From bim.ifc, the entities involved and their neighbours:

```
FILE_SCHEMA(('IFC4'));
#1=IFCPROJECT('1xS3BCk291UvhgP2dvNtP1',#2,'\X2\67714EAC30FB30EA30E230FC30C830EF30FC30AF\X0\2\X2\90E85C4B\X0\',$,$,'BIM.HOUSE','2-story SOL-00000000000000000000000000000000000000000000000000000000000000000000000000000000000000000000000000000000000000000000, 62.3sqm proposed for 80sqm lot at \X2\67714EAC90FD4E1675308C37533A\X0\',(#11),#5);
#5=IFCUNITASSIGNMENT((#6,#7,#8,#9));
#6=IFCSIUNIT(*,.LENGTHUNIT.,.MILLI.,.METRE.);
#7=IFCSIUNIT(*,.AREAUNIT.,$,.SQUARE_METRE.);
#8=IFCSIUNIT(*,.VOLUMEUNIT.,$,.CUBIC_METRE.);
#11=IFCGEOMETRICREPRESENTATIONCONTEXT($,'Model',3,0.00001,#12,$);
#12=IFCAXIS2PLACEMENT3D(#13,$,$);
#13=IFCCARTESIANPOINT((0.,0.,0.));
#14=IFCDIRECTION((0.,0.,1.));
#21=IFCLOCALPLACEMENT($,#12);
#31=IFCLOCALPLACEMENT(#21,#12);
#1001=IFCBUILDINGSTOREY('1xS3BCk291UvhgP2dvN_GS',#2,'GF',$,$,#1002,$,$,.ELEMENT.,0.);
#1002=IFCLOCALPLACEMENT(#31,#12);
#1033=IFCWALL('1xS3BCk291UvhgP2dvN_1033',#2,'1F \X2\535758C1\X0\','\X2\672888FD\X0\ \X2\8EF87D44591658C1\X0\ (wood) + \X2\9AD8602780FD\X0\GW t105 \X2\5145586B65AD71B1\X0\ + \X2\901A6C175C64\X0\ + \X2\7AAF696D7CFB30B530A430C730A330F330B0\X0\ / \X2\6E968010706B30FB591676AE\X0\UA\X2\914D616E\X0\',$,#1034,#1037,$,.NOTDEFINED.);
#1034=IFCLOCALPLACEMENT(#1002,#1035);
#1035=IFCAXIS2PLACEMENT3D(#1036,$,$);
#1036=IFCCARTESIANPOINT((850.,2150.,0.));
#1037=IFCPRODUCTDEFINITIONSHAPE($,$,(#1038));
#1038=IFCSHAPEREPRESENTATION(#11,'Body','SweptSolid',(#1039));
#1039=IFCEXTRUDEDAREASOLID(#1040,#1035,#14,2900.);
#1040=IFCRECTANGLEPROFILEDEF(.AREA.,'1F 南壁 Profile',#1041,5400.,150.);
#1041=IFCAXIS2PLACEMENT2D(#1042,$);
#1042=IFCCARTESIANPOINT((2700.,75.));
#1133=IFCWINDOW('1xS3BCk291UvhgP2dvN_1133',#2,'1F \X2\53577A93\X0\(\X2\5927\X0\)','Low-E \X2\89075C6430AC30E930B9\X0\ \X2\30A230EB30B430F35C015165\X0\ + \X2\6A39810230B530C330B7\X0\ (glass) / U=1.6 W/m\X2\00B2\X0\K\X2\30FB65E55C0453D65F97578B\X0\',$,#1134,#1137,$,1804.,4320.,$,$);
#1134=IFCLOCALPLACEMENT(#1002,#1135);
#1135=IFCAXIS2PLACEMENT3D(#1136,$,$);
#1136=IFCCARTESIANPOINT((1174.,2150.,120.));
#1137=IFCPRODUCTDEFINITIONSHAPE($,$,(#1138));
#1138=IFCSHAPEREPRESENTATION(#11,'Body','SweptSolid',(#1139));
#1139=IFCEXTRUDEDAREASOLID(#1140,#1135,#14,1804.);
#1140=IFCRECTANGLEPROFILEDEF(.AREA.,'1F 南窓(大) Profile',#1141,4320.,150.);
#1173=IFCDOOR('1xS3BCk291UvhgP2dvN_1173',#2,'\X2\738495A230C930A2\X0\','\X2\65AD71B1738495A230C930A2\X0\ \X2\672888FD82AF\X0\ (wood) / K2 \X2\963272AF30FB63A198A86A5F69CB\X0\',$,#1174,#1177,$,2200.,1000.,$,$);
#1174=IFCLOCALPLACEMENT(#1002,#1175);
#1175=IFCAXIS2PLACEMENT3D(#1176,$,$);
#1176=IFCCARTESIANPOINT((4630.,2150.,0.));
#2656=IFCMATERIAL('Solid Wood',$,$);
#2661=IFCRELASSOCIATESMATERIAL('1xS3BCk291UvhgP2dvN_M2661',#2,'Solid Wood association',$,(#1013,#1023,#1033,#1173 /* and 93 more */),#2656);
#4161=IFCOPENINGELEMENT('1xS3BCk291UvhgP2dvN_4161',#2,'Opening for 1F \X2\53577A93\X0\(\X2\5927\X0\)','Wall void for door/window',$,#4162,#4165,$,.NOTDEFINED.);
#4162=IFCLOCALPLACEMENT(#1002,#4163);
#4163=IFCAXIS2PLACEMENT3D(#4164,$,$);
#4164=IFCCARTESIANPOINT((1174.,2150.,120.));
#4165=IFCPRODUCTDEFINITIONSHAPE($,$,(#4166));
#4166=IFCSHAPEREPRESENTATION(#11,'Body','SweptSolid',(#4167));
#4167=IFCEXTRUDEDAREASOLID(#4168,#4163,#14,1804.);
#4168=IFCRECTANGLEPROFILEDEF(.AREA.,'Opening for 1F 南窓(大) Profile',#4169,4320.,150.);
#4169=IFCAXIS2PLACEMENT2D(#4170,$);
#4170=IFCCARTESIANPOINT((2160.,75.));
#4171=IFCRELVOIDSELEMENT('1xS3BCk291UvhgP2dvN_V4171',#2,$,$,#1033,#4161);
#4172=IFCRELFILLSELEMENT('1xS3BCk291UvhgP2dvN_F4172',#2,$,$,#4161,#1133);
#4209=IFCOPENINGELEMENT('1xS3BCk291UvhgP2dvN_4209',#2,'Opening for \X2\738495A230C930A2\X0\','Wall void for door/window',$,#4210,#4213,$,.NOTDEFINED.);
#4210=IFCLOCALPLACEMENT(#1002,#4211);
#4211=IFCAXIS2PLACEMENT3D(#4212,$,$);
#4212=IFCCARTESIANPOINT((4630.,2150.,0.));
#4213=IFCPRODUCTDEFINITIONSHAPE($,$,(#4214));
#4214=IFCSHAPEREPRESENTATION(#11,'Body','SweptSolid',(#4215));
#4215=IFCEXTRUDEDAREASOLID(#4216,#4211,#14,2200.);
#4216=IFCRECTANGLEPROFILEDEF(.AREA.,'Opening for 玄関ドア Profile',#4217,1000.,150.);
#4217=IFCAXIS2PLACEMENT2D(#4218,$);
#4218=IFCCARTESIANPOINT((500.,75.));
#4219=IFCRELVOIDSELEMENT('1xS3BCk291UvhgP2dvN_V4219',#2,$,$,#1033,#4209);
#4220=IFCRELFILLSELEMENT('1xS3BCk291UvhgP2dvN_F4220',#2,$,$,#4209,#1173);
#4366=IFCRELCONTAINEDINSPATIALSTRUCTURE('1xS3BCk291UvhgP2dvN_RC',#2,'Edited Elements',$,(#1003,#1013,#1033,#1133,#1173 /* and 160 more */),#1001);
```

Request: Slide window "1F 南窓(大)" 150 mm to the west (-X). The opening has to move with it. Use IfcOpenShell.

```python
import ifcopenshell
import ifcopenshell.api.geometry
import ifcopenshell.util.placement

model = ifcopenshell.open("bim.ifc")

window = model.by_guid("1xS3BCk291UvhgP2dvN_1133")
opening = window.FillsVoids[0].RelatingOpeningElement
wall = opening.VoidsElements[0].RelatingBuildingElement

wall_matrix = ifcopenshell.util.placement.get_local_placement(wall.ObjectPlacement)
shift = wall_matrix[:3, 0] * -150.0
before = ifcopenshell.util.placement.get_local_placement(window.ObjectPlacement)[:3, 3].copy()

# The window is not placed relative to its opening, so move both.
for product in (opening, window):
    matrix = ifcopenshell.util.placement.get_local_placement(product.ObjectPlacement)
    matrix[:3, 3] += shift
    ifcopenshell.api.geometry.edit_object_placement(model, product=product, matrix=matrix, is_si=False)

after = ifcopenshell.util.placement.get_local_placement(window.ObjectPlacement)[:3, 3]
print("window moved by", (after - before).round(3) + 0.0)

model.write("bim_updated.ifc")
```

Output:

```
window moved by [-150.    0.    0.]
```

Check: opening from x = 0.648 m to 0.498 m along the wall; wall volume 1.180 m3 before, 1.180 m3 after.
